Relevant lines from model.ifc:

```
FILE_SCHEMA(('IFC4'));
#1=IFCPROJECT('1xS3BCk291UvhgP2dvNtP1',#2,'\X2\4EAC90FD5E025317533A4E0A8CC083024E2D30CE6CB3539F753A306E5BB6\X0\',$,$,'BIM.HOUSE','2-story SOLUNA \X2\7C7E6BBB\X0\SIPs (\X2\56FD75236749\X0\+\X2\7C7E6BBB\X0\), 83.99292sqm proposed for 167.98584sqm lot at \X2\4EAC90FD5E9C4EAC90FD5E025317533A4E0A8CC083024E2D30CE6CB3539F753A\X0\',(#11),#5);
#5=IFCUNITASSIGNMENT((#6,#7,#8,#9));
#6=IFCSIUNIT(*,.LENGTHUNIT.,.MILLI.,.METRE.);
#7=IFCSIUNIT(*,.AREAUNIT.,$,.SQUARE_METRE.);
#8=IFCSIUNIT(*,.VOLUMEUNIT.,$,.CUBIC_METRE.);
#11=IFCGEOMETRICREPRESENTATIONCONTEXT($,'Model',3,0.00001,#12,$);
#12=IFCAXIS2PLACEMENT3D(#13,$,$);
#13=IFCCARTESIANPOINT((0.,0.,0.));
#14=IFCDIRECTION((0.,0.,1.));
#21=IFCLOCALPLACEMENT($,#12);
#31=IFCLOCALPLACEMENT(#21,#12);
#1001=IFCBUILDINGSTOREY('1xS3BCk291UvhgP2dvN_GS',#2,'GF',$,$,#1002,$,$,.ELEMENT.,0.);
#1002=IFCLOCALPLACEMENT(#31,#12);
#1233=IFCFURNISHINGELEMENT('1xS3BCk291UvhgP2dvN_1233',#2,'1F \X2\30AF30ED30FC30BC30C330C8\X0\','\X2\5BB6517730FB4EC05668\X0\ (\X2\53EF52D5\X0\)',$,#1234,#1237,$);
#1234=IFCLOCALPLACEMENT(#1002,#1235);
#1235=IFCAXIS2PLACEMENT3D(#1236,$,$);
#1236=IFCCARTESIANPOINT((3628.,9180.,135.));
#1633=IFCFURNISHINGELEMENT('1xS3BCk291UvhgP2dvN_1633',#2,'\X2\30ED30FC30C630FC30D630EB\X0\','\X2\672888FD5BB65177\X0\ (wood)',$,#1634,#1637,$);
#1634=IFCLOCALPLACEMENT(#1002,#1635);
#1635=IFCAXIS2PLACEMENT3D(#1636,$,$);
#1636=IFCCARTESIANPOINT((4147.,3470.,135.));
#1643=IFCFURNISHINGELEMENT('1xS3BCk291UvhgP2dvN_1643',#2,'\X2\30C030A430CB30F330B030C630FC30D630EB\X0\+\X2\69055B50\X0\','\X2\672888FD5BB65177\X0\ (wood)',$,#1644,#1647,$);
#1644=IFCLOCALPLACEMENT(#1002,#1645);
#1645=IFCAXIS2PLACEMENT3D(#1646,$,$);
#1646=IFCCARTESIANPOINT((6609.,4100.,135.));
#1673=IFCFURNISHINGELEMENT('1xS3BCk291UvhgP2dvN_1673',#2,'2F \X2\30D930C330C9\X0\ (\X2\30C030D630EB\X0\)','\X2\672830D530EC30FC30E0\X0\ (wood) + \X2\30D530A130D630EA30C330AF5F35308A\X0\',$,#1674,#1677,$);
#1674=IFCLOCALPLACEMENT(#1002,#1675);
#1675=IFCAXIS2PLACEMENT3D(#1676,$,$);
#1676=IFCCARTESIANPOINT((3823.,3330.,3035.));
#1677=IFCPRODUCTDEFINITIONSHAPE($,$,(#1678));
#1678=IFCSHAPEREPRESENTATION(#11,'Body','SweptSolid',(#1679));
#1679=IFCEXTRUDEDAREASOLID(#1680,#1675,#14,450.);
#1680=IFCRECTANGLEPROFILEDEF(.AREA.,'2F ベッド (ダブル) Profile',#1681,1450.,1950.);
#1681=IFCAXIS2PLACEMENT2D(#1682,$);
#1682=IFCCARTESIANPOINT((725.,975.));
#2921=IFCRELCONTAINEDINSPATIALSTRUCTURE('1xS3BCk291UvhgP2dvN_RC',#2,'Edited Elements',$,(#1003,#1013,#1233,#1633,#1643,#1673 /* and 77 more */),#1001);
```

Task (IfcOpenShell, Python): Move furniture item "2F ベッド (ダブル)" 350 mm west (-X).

```python
import ifcopenshell
import ifcopenshell.api.geometry
import ifcopenshell.util.placement
import ifcopenshell.util.unit

model = ifcopenshell.open("model.ifc")
unit_scale = ifcopenshell.util.unit.calculate_unit_scale(model)

item = model.by_guid("1xS3BCk291UvhgP2dvN_1673")
matrix = ifcopenshell.util.placement.get_local_placement(item.ObjectPlacement)
matrix[0, 3] -= 0.35 / unit_scale
ifcopenshell.api.geometry.edit_object_placement(model, product=item, matrix=matrix, is_si=False)

print(ifcopenshell.util.placement.get_local_placement(item.ObjectPlacement).round(3) + 0.0)

model.write("model_v2.ifc")
```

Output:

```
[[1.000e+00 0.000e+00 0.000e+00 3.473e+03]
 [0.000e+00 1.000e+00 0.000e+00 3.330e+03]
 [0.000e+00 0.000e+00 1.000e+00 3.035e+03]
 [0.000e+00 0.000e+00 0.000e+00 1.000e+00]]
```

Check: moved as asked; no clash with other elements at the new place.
